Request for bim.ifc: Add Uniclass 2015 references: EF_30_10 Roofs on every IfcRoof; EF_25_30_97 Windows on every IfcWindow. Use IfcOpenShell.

First a look at what the model holds.

```python
import ifcopenshell

model = ifcopenshell.open("bim.ifc")
print(model.schema)
print("classifications:", [c.Name for c in model.by_type("IfcClassification")])
for ifc_class in ("IfcDoor", "IfcRoof", "IfcStair", "IfcWall", "IfcWindow"):
    print(ifc_class, len(model.by_type(ifc_class)))
```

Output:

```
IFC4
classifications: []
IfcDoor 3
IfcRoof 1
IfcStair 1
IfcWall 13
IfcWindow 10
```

```python
import ifcopenshell
import ifcopenshell.api.classification

model = ifcopenshell.open("bim.ifc")

system = ifcopenshell.api.classification.add_classification(model, classification="Uniclass 2015")

codes = {
    "IfcRoof": ("EF_30_10", "Roofs"),
    "IfcWindow": ("EF_25_30_97", "Windows"),
}
for ifc_class, (code, name) in codes.items():
    products = model.by_type(ifc_class)
    ifcopenshell.api.classification.add_reference(
        model, products=products, classification=system, identification=code, name=name
    )
    print(code, len(products))

model.write("bim_rev.ifc")
```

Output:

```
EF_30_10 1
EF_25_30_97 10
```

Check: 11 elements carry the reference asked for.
